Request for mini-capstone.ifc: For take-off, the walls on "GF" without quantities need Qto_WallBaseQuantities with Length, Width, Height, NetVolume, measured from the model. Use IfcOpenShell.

First a look at what the model holds.

```python
import ifcopenshell
import ifcopenshell.util.element
import ifcopenshell.util.unit

model = ifcopenshell.open("mini-capstone.ifc")
print(model.schema)
for unit_type in ("LENGTHUNIT", "AREAUNIT", "VOLUMEUNIT"):
    print(unit_type, ifcopenshell.util.unit.calculate_unit_scale(model, unit_type))
storey = next(s for s in model.by_type("IfcBuildingStorey") if s.Name == "GF")
walls = [e for e in ifcopenshell.util.element.get_decomposition(storey) if e.is_a("IfcWall")]
for e in sorted(walls, key=lambda e: e.id()):
    print(e.id(), e.is_a(), e.Name, list(ifcopenshell.util.element.get_psets(e, qtos_only=True)), sep=" | ")
```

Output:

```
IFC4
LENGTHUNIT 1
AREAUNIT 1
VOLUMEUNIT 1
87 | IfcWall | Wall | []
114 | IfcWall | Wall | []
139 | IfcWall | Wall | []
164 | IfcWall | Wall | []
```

```python
import ifcopenshell
import ifcopenshell.api.pset
import ifcopenshell.geom
import ifcopenshell.util.element
import ifcopenshell.util.shape
import ifcopenshell.util.unit

model = ifcopenshell.open("mini-capstone.ifc")
unit_scale = ifcopenshell.util.unit.calculate_unit_scale(model)
volume_scale = ifcopenshell.util.unit.calculate_unit_scale(model, "VOLUMEUNIT")
settings = ifcopenshell.geom.settings()

storey = next(s for s in model.by_type("IfcBuildingStorey") if s.Name == "GF")
walls = [e for e in ifcopenshell.util.element.get_decomposition(storey) if e.is_a("IfcWall")]

for e in sorted(walls, key=lambda e: e.id()):
    if ifcopenshell.util.element.get_psets(e, qtos_only=True, should_inherit=False):
        continue
    # Geometry comes back in metres, in the element's own axes.
    shape = ifcopenshell.geom.create_shape(settings, e)
    values = {
        "Length": ifcopenshell.util.shape.get_x(shape.geometry) / unit_scale,
        "Width": ifcopenshell.util.shape.get_y(shape.geometry) / unit_scale,
        "Height": ifcopenshell.util.shape.get_z(shape.geometry) / unit_scale,
        "NetVolume": ifcopenshell.util.shape.get_volume(shape.geometry) / volume_scale,
    }
    qto = ifcopenshell.api.pset.add_qto(model, product=e, name="Qto_WallBaseQuantities")
    ifcopenshell.api.pset.edit_qto(model, qto=qto, properties=values)
    print(e.id(), {k: round(v, 3) for k, v in values.items()})

model.write("mini-capstone_updated.ifc")
```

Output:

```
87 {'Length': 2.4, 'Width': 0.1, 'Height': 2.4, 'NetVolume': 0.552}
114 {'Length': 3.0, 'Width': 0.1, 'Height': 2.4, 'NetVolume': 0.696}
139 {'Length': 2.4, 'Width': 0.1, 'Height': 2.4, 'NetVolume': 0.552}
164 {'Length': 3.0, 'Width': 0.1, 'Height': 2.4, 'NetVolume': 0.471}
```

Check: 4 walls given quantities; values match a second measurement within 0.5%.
